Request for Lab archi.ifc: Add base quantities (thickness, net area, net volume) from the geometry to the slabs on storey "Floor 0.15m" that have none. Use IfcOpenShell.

First a look at what the model holds.

```python
import ifcopenshell
import ifcopenshell.util.element
import ifcopenshell.util.unit

model = ifcopenshell.open("Lab archi.ifc")
print(model.schema)
for unit_type in ("LENGTHUNIT", "AREAUNIT", "VOLUMEUNIT"):
    print(unit_type, ifcopenshell.util.unit.calculate_unit_scale(model, unit_type))
storey = next(s for s in model.by_type("IfcBuildingStorey") if s.Name == "Floor 0.15m")
slabs = [e for e in ifcopenshell.util.element.get_decomposition(storey) if e.is_a("IfcSlab")]
for e in sorted(slabs, key=lambda e: e.id()):
    print(e.id(), e.is_a(), e.Name, list(ifcopenshell.util.element.get_psets(e, qtos_only=True)), sep=" | ")
```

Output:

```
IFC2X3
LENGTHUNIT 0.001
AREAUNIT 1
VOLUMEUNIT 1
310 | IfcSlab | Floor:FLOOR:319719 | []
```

```python
import ifcopenshell
import ifcopenshell.api.pset
import ifcopenshell.geom
import ifcopenshell.util.element
import ifcopenshell.util.shape
import ifcopenshell.util.unit

model = ifcopenshell.open("Lab archi.ifc")
unit_scale = ifcopenshell.util.unit.calculate_unit_scale(model)
area_scale = ifcopenshell.util.unit.calculate_unit_scale(model, "AREAUNIT")
volume_scale = ifcopenshell.util.unit.calculate_unit_scale(model, "VOLUMEUNIT")
settings = ifcopenshell.geom.settings()

storey = next(s for s in model.by_type("IfcBuildingStorey") if s.Name == "Floor 0.15m")
slabs = [e for e in ifcopenshell.util.element.get_decomposition(storey) if e.is_a("IfcSlab")]

for e in sorted(slabs, key=lambda e: e.id()):
    if ifcopenshell.util.element.get_psets(e, qtos_only=True, should_inherit=False):
        continue
    # Geometry comes back in metres, in the element's own axes.
    shape = ifcopenshell.geom.create_shape(settings, e)
    values = {
        "Width": ifcopenshell.util.shape.get_z(shape.geometry) / unit_scale,
        "NetArea": ifcopenshell.util.shape.get_footprint_area(shape.geometry) / area_scale,
        "NetVolume": ifcopenshell.util.shape.get_volume(shape.geometry) / volume_scale,
    }
    qto = ifcopenshell.api.pset.add_qto(model, product=e, name="BaseQuantities")
    ifcopenshell.api.pset.edit_qto(model, qto=qto, properties=values)
    print(e.id(), {k: round(v, 3) for k, v in values.items()})

model.write("Lab archi_rev.ifc")
```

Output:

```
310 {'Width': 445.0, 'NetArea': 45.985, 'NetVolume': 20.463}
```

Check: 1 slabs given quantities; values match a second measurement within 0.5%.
